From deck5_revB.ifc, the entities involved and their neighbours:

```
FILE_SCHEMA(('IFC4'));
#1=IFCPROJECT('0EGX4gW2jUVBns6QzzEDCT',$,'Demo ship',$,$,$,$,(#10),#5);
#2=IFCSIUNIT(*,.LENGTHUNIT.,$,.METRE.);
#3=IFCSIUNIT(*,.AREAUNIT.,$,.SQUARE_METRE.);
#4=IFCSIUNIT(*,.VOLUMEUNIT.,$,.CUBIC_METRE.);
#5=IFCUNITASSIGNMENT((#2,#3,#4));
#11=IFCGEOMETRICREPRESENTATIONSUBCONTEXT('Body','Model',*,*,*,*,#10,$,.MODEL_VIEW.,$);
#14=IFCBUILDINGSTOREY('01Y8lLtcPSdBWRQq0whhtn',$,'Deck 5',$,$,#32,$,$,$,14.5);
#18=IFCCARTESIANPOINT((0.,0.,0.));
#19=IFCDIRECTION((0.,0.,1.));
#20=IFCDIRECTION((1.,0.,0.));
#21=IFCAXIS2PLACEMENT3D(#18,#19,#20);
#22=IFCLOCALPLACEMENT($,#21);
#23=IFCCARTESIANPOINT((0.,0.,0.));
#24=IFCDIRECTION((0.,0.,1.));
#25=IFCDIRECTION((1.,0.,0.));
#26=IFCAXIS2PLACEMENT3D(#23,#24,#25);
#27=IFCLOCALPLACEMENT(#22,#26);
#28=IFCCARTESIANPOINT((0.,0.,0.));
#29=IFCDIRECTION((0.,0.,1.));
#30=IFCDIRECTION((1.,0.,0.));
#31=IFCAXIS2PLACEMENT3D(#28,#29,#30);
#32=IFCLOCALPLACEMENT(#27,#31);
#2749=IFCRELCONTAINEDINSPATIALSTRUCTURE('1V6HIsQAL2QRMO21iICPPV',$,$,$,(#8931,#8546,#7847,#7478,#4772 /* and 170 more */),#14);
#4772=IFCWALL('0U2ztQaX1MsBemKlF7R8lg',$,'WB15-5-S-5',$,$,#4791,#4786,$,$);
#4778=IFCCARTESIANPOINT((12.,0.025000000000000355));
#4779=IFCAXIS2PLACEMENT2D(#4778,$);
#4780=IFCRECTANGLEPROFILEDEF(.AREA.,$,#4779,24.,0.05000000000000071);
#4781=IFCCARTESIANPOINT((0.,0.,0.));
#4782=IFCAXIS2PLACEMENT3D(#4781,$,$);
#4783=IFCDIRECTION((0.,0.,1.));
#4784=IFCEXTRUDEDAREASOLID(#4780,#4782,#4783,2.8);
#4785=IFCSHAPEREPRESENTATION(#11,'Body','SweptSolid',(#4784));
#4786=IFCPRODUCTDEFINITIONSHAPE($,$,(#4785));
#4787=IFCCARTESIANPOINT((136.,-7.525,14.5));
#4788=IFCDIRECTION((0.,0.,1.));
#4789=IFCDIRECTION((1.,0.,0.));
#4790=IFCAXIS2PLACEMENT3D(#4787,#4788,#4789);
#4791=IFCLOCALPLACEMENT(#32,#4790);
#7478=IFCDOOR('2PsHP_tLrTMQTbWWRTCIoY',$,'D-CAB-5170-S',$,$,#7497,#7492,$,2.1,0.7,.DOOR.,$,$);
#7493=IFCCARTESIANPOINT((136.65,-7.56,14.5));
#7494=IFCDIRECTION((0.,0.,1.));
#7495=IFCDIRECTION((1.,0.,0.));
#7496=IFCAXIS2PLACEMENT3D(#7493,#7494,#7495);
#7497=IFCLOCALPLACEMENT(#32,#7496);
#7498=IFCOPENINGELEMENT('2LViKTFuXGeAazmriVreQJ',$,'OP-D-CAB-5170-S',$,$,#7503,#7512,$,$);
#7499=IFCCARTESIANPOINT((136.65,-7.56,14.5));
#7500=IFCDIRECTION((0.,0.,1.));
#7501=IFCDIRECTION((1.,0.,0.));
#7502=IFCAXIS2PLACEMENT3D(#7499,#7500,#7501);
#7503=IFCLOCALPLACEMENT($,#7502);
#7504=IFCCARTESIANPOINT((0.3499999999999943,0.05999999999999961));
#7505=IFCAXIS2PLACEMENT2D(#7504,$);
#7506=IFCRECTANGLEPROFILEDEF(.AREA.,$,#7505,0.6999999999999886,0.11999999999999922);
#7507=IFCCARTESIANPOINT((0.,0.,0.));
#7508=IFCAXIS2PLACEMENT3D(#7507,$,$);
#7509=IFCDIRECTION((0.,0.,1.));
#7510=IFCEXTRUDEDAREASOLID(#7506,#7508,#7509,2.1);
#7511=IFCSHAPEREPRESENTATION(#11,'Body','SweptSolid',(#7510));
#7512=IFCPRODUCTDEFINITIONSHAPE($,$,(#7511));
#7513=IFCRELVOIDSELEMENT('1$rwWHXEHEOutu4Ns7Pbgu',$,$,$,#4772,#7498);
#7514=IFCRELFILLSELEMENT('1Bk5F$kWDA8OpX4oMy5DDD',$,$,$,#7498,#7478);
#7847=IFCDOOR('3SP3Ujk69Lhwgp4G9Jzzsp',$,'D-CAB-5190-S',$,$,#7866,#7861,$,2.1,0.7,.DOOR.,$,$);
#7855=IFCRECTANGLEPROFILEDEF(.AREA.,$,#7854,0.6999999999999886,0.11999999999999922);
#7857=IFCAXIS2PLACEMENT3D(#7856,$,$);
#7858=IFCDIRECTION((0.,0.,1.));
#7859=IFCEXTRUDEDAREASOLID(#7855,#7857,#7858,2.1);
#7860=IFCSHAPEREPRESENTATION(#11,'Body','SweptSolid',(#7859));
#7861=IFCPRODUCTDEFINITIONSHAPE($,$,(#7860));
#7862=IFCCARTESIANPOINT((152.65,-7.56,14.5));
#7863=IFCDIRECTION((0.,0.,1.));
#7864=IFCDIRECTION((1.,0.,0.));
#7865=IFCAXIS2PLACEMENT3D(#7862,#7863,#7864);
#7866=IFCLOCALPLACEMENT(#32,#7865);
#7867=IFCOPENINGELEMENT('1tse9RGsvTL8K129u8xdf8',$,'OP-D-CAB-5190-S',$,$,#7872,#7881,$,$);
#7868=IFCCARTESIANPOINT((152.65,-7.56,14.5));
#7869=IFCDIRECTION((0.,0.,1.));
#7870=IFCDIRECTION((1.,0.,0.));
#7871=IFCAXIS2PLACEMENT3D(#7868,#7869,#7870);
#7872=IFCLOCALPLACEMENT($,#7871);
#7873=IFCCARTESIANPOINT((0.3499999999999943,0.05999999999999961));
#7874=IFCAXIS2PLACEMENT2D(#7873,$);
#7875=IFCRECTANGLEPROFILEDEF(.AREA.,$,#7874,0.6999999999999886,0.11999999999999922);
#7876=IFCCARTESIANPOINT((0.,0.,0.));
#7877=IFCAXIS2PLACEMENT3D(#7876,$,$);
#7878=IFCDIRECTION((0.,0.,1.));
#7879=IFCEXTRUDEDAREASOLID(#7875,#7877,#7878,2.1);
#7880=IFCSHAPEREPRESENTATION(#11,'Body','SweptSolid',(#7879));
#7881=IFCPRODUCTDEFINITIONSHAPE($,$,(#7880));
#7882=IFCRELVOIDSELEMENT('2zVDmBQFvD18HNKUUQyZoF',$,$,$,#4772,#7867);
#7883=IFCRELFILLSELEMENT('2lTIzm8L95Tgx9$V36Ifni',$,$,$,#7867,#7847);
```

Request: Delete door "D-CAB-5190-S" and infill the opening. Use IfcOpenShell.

```python
import ifcopenshell
import ifcopenshell.api.feature
import ifcopenshell.api.root
import ifcopenshell.geom
import ifcopenshell.util.shape

model = ifcopenshell.open("deck5_revB.ifc")
settings = ifcopenshell.geom.settings()


def volume(element):
    """Net volume in cubic metres, openings subtracted."""
    shape = ifcopenshell.geom.create_shape(settings, element)
    return ifcopenshell.util.shape.get_volume(shape.geometry)


door = model.by_guid("3SP3Ujk69Lhwgp4G9Jzzsp")
opening = door.FillsVoids[0].RelatingOpeningElement
wall = opening.VoidsElements[0].RelatingBuildingElement
before = volume(wall)

ifcopenshell.api.root.remove_product(model, product=door)
ifcopenshell.api.feature.remove_feature(model, feature=opening)

after = volume(wall)

print(f"wall volume {before:.3f} -> {after:.3f} m3")

model.write("deck5_revB_updated.ifc")
```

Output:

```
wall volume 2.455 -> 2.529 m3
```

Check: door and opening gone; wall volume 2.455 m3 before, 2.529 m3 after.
